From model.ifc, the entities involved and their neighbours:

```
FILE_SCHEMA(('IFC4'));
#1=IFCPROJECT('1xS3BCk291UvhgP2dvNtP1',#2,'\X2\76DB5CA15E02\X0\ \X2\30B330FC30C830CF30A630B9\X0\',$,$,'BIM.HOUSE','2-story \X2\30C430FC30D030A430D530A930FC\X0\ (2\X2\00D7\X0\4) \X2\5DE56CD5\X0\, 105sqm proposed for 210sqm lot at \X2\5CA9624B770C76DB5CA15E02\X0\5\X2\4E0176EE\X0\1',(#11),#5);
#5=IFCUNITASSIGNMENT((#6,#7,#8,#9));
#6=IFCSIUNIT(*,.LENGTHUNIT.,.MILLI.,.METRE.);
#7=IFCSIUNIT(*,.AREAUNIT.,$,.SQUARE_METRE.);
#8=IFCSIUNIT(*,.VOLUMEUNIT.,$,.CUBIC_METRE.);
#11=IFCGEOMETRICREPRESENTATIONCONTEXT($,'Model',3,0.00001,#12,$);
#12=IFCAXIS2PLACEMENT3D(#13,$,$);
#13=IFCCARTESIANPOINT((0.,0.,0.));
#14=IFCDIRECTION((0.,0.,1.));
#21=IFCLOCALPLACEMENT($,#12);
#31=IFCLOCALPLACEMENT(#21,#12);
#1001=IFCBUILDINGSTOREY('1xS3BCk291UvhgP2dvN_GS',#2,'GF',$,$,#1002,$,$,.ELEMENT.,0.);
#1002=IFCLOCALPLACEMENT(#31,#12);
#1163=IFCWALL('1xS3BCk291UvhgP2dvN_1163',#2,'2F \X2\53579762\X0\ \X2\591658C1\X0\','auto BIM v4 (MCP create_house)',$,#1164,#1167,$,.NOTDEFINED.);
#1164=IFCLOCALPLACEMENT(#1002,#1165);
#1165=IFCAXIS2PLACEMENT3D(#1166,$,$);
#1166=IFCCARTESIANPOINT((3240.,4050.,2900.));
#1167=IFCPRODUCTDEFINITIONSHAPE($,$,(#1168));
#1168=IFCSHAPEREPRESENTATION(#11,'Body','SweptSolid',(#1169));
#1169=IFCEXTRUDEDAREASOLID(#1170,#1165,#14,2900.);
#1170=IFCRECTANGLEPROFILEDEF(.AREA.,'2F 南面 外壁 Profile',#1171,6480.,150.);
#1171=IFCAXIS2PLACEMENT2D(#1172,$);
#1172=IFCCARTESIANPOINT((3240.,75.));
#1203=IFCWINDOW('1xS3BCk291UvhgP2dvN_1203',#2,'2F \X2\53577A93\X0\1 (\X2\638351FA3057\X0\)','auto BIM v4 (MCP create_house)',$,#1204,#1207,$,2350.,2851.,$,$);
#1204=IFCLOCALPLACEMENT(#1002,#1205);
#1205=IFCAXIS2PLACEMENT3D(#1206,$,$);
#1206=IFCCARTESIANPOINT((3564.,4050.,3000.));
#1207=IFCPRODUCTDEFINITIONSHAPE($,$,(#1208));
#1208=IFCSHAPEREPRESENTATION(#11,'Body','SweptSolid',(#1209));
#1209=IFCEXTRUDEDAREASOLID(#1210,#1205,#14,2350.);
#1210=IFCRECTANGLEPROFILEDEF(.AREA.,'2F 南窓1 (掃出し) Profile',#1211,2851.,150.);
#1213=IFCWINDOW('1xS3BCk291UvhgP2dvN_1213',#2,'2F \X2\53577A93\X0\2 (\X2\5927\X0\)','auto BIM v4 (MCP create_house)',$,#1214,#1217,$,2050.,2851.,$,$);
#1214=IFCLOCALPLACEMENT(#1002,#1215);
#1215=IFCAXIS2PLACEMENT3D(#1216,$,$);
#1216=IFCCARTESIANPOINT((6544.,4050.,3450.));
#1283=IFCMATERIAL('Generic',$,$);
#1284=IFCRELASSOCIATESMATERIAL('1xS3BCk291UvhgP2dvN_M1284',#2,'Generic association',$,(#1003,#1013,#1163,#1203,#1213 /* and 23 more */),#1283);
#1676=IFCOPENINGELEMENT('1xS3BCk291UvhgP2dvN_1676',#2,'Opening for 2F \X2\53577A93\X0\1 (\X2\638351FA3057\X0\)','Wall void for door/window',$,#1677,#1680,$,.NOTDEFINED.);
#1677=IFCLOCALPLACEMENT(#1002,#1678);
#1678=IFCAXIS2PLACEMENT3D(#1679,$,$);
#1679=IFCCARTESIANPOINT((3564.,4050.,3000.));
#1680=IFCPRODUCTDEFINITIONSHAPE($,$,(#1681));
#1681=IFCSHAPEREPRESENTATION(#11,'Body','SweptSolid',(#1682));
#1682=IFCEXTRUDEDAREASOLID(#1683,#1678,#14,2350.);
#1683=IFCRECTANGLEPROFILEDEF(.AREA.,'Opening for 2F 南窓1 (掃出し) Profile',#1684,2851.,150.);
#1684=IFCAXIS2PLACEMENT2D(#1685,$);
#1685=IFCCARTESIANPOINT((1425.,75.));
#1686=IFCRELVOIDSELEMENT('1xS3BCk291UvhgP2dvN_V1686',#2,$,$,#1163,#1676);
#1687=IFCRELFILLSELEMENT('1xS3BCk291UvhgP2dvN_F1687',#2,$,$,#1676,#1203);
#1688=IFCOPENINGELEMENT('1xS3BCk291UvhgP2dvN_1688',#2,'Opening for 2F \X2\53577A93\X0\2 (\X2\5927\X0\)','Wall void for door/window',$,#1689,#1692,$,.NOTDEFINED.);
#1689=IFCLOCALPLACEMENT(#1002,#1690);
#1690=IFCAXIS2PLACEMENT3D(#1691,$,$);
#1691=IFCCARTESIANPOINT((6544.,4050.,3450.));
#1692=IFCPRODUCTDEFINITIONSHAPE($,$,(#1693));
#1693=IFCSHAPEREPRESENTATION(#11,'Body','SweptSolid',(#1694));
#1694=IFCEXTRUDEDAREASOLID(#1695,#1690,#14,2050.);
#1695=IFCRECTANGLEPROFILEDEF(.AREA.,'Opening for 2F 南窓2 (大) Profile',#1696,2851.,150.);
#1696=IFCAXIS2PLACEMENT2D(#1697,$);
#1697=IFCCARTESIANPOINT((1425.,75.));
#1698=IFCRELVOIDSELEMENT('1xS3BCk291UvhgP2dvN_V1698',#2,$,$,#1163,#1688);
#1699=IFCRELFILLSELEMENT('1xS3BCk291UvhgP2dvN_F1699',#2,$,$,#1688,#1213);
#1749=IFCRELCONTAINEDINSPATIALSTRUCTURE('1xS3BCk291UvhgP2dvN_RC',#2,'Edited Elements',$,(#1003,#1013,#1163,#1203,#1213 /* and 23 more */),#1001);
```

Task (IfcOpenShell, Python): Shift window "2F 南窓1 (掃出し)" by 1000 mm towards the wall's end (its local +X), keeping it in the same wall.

```python
import ifcopenshell
import ifcopenshell.api.geometry
import ifcopenshell.util.placement
import ifcopenshell.util.unit

model = ifcopenshell.open("model.ifc")
unit_scale = ifcopenshell.util.unit.calculate_unit_scale(model)

window = model.by_id(1203)
opening = window.FillsVoids[0].RelatingOpeningElement
wall = opening.VoidsElements[0].RelatingBuildingElement

wall_matrix = ifcopenshell.util.placement.get_local_placement(wall.ObjectPlacement)
shift = wall_matrix[:3, 0] * 1 / unit_scale
before = ifcopenshell.util.placement.get_local_placement(window.ObjectPlacement)[:3, 3].copy()

# The window is not placed relative to its opening, so move both.
for product in (opening, window):
    matrix = ifcopenshell.util.placement.get_local_placement(product.ObjectPlacement)
    matrix[:3, 3] += shift
    ifcopenshell.api.geometry.edit_object_placement(model, product=product, matrix=matrix, is_si=False)

after = ifcopenshell.util.placement.get_local_placement(window.ObjectPlacement)[:3, 3]
print("window moved by", (after - before).round(3) + 0.0)

model.write("model_rev.ifc")
```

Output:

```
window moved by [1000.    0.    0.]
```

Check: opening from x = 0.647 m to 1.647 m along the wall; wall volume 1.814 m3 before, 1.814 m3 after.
